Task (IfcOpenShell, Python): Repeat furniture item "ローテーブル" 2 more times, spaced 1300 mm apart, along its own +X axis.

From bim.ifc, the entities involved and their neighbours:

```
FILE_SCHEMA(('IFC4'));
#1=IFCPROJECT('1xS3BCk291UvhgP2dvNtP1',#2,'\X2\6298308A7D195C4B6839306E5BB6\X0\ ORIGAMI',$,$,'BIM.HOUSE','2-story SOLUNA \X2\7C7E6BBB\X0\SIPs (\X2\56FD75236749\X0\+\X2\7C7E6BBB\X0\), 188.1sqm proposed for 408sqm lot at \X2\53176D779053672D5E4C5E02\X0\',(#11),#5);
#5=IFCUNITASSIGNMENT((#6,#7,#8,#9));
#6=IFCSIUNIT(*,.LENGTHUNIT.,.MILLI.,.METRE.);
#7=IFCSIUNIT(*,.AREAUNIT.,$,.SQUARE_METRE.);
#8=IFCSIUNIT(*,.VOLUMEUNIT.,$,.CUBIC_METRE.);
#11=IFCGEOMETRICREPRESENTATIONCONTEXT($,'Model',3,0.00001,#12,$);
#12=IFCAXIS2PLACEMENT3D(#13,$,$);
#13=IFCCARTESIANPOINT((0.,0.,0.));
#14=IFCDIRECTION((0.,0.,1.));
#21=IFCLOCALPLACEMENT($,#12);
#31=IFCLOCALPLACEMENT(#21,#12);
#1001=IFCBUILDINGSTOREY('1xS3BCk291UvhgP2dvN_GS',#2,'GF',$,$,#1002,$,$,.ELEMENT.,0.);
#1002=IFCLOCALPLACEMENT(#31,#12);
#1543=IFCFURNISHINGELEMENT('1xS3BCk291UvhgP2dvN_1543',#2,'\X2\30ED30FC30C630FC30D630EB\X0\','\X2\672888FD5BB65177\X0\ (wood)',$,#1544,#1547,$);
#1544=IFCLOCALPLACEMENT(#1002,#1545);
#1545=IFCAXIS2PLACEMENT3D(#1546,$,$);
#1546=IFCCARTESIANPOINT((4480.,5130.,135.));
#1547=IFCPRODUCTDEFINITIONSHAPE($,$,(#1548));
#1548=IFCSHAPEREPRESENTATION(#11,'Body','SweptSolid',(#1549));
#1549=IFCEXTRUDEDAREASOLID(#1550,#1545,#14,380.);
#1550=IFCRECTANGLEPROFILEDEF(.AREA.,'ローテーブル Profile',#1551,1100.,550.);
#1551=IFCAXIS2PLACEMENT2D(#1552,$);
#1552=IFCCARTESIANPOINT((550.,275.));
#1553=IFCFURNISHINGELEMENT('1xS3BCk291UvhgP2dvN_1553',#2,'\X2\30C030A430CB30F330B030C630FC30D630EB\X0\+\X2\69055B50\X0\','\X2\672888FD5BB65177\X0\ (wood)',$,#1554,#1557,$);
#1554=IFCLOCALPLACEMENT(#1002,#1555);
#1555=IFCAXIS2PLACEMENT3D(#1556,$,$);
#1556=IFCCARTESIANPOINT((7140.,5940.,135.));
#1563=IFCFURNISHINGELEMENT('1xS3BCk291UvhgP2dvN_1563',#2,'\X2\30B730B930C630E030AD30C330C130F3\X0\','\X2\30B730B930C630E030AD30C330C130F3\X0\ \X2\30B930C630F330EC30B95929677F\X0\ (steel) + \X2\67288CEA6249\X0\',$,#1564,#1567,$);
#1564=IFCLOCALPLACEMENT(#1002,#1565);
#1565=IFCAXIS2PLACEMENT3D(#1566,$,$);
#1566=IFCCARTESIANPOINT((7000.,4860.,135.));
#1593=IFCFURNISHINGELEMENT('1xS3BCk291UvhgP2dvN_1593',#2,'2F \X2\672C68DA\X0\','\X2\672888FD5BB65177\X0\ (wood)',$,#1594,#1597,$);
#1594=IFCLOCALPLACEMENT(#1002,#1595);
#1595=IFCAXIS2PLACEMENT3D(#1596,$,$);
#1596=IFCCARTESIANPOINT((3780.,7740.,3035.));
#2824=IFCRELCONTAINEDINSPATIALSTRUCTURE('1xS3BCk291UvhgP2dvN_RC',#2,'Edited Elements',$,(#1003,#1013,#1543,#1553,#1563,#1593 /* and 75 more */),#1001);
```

```python
import ifcopenshell
import ifcopenshell.api.geometry
import ifcopenshell.api.root
import ifcopenshell.util.element
import ifcopenshell.util.placement

model = ifcopenshell.open("bim.ifc")


def reuse_history(source, copy):
    """copy_class also copies each property set's owner history, people and application; keep the originals."""
    for rel in copy.IsDefinedBy:
        if rel.is_a("IfcRelDefinesByProperties") and (history := rel.RelatingPropertyDefinition.OwnerHistory):
            rel.RelatingPropertyDefinition.OwnerHistory = source.OwnerHistory
            ifcopenshell.util.element.remove_deep2(model, history)


source = model.by_id(1543)
base = ifcopenshell.util.placement.get_local_placement(source.ObjectPlacement)
step = base[:3, 0] * 1300.0

for i in range(1, 3):
    copy = ifcopenshell.api.root.copy_class(model, product=source)
    copy.Representation = ifcopenshell.util.element.copy_deep(
        model, source.Representation, exclude=["IfcGeometricRepresentationContext", "IfcRepresentationMap"]
    )
    reuse_history(source, copy)
    matrix = base.copy()
    matrix[:3, 3] += i * step
    print("added at", matrix[:3, 3].round(3) + 0.0)
    ifcopenshell.api.geometry.edit_object_placement(model, product=copy, matrix=matrix, is_si=False)

model.write("bim-out.ifc")
```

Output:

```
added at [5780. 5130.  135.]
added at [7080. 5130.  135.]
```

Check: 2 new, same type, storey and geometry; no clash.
